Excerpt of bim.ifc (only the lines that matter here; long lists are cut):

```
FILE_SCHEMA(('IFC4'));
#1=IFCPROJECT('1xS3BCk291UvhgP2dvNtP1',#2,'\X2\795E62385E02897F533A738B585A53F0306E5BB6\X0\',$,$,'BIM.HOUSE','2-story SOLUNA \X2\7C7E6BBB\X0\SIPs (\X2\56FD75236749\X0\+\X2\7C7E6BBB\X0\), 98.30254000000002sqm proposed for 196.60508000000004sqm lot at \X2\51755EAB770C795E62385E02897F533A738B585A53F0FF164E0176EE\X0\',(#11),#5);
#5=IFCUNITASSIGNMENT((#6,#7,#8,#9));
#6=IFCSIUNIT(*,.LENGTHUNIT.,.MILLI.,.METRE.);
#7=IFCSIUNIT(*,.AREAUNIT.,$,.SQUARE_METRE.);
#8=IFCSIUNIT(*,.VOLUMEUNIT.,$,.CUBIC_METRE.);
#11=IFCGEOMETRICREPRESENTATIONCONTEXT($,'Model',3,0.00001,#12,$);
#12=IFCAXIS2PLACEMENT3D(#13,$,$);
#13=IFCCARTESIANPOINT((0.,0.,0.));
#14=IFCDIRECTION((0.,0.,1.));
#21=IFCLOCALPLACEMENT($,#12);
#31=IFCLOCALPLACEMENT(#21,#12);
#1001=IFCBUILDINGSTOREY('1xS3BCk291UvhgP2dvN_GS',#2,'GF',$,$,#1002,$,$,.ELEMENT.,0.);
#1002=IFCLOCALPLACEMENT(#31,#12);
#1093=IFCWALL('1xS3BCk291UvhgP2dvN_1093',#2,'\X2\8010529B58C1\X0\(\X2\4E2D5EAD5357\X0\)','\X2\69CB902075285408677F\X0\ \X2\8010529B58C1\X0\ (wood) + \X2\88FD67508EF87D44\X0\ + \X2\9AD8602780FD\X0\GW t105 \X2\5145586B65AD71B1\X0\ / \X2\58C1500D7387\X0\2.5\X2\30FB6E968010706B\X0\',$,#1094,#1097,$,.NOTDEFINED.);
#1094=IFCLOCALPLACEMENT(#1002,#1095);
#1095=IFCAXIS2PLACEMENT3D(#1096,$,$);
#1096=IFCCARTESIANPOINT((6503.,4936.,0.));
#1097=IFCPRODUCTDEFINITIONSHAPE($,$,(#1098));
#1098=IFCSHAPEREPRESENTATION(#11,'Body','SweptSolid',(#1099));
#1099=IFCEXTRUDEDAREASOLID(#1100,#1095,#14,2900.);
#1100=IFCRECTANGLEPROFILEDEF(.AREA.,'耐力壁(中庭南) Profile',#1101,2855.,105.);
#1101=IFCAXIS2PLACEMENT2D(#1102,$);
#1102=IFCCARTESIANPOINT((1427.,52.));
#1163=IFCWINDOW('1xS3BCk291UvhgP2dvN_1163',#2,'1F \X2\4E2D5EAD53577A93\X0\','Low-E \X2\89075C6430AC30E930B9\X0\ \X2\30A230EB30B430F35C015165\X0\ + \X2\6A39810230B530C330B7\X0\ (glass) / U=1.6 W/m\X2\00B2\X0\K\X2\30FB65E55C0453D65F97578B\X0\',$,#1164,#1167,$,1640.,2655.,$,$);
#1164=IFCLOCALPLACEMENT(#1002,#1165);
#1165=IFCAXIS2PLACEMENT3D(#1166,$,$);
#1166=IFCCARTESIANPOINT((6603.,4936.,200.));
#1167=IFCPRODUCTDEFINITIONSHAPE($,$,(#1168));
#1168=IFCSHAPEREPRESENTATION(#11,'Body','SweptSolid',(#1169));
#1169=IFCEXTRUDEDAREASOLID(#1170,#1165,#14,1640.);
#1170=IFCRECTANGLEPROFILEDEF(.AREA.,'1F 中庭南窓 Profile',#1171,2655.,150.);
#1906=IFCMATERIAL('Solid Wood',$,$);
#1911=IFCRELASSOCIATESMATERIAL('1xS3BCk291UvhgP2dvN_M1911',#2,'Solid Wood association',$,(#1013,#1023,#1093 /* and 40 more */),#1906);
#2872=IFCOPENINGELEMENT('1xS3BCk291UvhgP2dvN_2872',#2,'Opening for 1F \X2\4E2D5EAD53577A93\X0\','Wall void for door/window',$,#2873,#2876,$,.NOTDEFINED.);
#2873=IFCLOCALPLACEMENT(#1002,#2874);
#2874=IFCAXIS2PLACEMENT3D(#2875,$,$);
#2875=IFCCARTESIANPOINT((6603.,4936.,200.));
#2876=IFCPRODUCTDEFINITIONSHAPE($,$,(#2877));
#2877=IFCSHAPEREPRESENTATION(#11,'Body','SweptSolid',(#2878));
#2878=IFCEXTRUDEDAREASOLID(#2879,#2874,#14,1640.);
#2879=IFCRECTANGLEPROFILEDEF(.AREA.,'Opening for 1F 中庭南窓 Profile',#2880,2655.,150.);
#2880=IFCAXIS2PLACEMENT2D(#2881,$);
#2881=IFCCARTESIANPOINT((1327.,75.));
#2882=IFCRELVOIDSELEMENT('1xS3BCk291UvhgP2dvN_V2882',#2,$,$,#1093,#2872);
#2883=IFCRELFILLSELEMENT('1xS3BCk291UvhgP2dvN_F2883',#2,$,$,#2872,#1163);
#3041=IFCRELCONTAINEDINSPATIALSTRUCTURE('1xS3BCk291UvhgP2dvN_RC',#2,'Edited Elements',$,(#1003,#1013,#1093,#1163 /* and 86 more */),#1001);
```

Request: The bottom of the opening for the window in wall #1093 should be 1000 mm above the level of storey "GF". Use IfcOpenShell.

```python
import numpy as np
import ifcopenshell
import ifcopenshell.api.geometry
import ifcopenshell.geom
import ifcopenshell.util.element
import ifcopenshell.util.placement
import ifcopenshell.util.shape
import ifcopenshell.util.unit

model = ifcopenshell.open("bim.ifc")
unit_scale = ifcopenshell.util.unit.calculate_unit_scale(model)

window = model.by_guid("1xS3BCk291UvhgP2dvN_1163")
opening = window.FillsVoids[0].RelatingOpeningElement
storey = ifcopenshell.util.element.get_container(window, ifc_class="IfcBuildingStorey")
level = ifcopenshell.util.placement.get_local_placement(storey.ObjectPlacement)[2, 3]

# The opening's origin need not be at the sill, so measure its lowest point.
shape = ifcopenshell.geom.create_shape(ifcopenshell.geom.settings(), opening)
bottom = ifcopenshell.util.shape.get_shape_bottom_elevation(shape, shape.geometry) / unit_scale
dz = level + 1000.0 - bottom

shift = np.array([0.0, 0.0, dz])
# The window is not placed relative to its opening, so move both.
for product in (opening, window):
    matrix = ifcopenshell.util.placement.get_local_placement(product.ObjectPlacement)
    matrix[:3, 3] += shift
    ifcopenshell.api.geometry.edit_object_placement(model, product=product, matrix=matrix, is_si=False)

print(f"moved by {dz * unit_scale:+.3f} m")

model.write("bim-out.ifc")
```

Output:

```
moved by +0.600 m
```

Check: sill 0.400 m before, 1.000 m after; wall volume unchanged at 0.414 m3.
